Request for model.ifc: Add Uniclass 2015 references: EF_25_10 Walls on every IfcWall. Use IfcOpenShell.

First a look at what the model holds.

```python
import ifcopenshell

model = ifcopenshell.open("model.ifc")
print(model.schema)
print("classifications:", [c.Name for c in model.by_type("IfcClassification")])
for ifc_class in ("IfcDoor", "IfcRoof", "IfcStair", "IfcWall", "IfcWindow"):
    print(ifc_class, len(model.by_type(ifc_class)))
```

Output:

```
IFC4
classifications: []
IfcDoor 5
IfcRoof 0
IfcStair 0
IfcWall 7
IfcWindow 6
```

```python
import ifcopenshell
import ifcopenshell.api.classification

model = ifcopenshell.open("model.ifc")

system = ifcopenshell.api.classification.add_classification(model, classification="Uniclass 2015")

codes = {
    "IfcWall": ("EF_25_10", "Walls"),
}
for ifc_class, (code, name) in codes.items():
    products = model.by_type(ifc_class)
    ifcopenshell.api.classification.add_reference(
        model, products=products, classification=system, identification=code, name=name
    )
    print(code, len(products))

model.write("model_rev.ifc")
```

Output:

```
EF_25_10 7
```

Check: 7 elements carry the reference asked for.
